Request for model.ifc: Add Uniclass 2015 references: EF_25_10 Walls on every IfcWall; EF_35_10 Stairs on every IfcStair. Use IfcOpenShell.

First a look at what the model holds.

```python
import ifcopenshell

model = ifcopenshell.open("model.ifc")
print(model.schema)
print("classifications:", [c.Name for c in model.by_type("IfcClassification")])
for ifc_class in ("IfcDoor", "IfcRoof", "IfcStair", "IfcWall", "IfcWindow"):
    print(ifc_class, len(model.by_type(ifc_class)))
```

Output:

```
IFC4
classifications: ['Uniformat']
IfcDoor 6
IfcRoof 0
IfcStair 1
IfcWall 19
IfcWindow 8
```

```python
import ifcopenshell
import ifcopenshell.api.classification

model = ifcopenshell.open("model.ifc")

system = ifcopenshell.api.classification.add_classification(model, classification="Uniclass 2015")

codes = {
    "IfcWall": ("EF_25_10", "Walls"),
    "IfcStair": ("EF_35_10", "Stairs"),
}
for ifc_class, (code, name) in codes.items():
    products = model.by_type(ifc_class)
    ifcopenshell.api.classification.add_reference(
        model, products=products, classification=system, identification=code, name=name
    )
    print(code, len(products))

model.write("model_updated.ifc")
```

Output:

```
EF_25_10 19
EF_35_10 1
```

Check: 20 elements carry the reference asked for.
